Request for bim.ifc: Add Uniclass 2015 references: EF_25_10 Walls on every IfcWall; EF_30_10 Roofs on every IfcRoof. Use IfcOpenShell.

First a look at what the model holds.

```python
import ifcopenshell

model = ifcopenshell.open("bim.ifc")
print(model.schema)
print("classifications:", [c.Name for c in model.by_type("IfcClassification")])
for ifc_class in ("IfcDoor", "IfcRoof", "IfcStair", "IfcWall", "IfcWindow"):
    print(ifc_class, len(model.by_type(ifc_class)))
```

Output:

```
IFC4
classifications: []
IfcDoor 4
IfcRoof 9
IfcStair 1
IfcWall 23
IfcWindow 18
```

```python
import ifcopenshell
import ifcopenshell.api.classification

model = ifcopenshell.open("bim.ifc")

system = ifcopenshell.api.classification.add_classification(model, classification="Uniclass 2015")

codes = {
    "IfcWall": ("EF_25_10", "Walls"),
    "IfcRoof": ("EF_30_10", "Roofs"),
}
for ifc_class, (code, name) in codes.items():
    products = model.by_type(ifc_class)
    ifcopenshell.api.classification.add_reference(
        model, products=products, classification=system, identification=code, name=name
    )
    print(code, len(products))

model.write("bim_updated.ifc")
```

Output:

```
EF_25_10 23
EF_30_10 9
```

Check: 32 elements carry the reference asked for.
